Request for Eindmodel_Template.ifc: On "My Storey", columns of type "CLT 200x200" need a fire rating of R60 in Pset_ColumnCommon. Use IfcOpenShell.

First a look at what the model holds.

```python
import ifcopenshell
import ifcopenshell.util.element

model = ifcopenshell.open("Eindmodel_Template.ifc")
print(model.schema)
storey = next(s for s in model.by_type("IfcBuildingStorey") if s.Name == "My Storey")
columns = [e for e in ifcopenshell.util.element.get_decomposition(storey) if e.is_a("IfcColumn")]
seen = {}
for e in columns:
    element_type = ifcopenshell.util.element.get_type(e)
    key = (element_type.Name if element_type != e and element_type else None, ifcopenshell.util.element.get_pset(e, "Pset_ColumnCommon", "FireRating"))
    seen[key] = seen.get(key, 0) + 1
for (name, value), count in sorted(seen.items(), key=str):
    print(count, "x", name, "|", value)
```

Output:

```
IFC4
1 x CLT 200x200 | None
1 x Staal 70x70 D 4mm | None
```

```python
import ifcopenshell
import ifcopenshell.api.pset
import ifcopenshell.util.element

model = ifcopenshell.open("Eindmodel_Template.ifc")

storey = next(s for s in model.by_type("IfcBuildingStorey") if s.Name == "My Storey")
columns = [e for e in ifcopenshell.util.element.get_decomposition(storey) if e.is_a("IfcColumn")]

count = 0
for e in columns:
    element_type = ifcopenshell.util.element.get_type(e)
    if element_type in (None, e) or element_type.Name != "CLT 200x200":
        continue
    # add_pset returns the element's existing set when there is one.
    pset = ifcopenshell.api.pset.add_pset(model, product=e, name="Pset_ColumnCommon")
    ifcopenshell.api.pset.edit_pset(model, pset=pset, properties={"FireRating": "R60"})
    count += 1

print(count, "columns updated")

model.write("Eindmodel_Template-out.ifc")
```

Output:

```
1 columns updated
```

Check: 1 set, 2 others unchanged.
